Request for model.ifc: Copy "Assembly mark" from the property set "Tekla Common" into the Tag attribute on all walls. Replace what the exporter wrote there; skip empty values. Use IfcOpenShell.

First a look at what the model holds.

```python
import ifcopenshell
import ifcopenshell.util.element

model = ifcopenshell.open("model.ifc")
print(model.schema)
walls = model.by_type("IfcWall")
print(len(walls), "walls")
for e in walls[:8]:
    source = ifcopenshell.util.element.get_pset(e, "Tekla Common", "Assembly mark")
    target = e.Tag
    print(e.id(), repr(source), repr(target), sep=" | ")
```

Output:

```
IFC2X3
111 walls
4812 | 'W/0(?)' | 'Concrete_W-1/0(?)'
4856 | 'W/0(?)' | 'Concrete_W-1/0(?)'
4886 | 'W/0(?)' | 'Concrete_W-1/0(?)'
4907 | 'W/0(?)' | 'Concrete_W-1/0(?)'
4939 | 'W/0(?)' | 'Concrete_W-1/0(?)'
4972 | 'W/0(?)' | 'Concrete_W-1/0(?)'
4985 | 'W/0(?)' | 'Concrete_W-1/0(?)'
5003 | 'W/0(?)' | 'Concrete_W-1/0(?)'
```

```python
import ifcopenshell
import ifcopenshell.util.element

model = ifcopenshell.open("model.ifc")

count = 0
for e in model.by_type("IfcWall"):
    value = ifcopenshell.util.element.get_pset(e, "Tekla Common", "Assembly mark")
    current = e.Tag
    if not value or not value.strip() or current == value:
        continue
    e.Tag = value
    count += 1

print(count, "walls updated")

model.write("model-out.ifc")
```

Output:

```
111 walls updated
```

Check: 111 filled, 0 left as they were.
